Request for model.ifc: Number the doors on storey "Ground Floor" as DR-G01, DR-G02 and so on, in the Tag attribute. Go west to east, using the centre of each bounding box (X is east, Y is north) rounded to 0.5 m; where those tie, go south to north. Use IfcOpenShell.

First a look at what the model holds.

```python
import ifcopenshell
import ifcopenshell.util.element
import ifcopenshell.util.placement

model = ifcopenshell.open("model.ifc")
print(model.schema)
storey = next(s for s in model.by_type("IfcBuildingStorey") if s.Name == "Ground Floor")
doors = [e for e in ifcopenshell.util.element.get_decomposition(storey) if e.is_a("IfcDoor")]
for e in sorted(doors, key=lambda e: e.id()):
    origin = ifcopenshell.util.placement.get_local_placement(e.ObjectPlacement)[:3, 3]
    print(e.id(), e.Tag, e.Name, origin.round(2) + 0.0, sep=" | ")
```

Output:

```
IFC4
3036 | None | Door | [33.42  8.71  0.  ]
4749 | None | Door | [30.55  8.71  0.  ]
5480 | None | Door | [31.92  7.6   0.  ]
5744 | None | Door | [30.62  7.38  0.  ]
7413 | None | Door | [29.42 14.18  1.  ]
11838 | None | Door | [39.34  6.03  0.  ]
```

```python
import ifcopenshell
import ifcopenshell.geom
import ifcopenshell.util.element
import ifcopenshell.util.shape

model = ifcopenshell.open("model.ifc")
settings = ifcopenshell.geom.settings()
settings.set("use-world-coords", True)


def centre(element):
    shape = ifcopenshell.geom.create_shape(settings, element)
    return ifcopenshell.util.shape.get_bbox_centroid(shape.geometry)


storey = next(s for s in model.by_type("IfcBuildingStorey") if s.Name == "Ground Floor")
doors = [e for e in ifcopenshell.util.element.get_decomposition(storey) if e.is_a("IfcDoor")]

# Insertion points can sit at a corner or the storey origin, so sort by the geometry (in metres).
centres = {e: centre(e) for e in doors}
doors.sort(key=lambda e: (round(centres[e][0] / 0.5), centres[e][1]))

for i, e in enumerate(doors, start=1):
    number = f"DR-G{i:02d}"
    e.Tag = number
    print(e.id(), number)

model.write("model_v2.ifc")
```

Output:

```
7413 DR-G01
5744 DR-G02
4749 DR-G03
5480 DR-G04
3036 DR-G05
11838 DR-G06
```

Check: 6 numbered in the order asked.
